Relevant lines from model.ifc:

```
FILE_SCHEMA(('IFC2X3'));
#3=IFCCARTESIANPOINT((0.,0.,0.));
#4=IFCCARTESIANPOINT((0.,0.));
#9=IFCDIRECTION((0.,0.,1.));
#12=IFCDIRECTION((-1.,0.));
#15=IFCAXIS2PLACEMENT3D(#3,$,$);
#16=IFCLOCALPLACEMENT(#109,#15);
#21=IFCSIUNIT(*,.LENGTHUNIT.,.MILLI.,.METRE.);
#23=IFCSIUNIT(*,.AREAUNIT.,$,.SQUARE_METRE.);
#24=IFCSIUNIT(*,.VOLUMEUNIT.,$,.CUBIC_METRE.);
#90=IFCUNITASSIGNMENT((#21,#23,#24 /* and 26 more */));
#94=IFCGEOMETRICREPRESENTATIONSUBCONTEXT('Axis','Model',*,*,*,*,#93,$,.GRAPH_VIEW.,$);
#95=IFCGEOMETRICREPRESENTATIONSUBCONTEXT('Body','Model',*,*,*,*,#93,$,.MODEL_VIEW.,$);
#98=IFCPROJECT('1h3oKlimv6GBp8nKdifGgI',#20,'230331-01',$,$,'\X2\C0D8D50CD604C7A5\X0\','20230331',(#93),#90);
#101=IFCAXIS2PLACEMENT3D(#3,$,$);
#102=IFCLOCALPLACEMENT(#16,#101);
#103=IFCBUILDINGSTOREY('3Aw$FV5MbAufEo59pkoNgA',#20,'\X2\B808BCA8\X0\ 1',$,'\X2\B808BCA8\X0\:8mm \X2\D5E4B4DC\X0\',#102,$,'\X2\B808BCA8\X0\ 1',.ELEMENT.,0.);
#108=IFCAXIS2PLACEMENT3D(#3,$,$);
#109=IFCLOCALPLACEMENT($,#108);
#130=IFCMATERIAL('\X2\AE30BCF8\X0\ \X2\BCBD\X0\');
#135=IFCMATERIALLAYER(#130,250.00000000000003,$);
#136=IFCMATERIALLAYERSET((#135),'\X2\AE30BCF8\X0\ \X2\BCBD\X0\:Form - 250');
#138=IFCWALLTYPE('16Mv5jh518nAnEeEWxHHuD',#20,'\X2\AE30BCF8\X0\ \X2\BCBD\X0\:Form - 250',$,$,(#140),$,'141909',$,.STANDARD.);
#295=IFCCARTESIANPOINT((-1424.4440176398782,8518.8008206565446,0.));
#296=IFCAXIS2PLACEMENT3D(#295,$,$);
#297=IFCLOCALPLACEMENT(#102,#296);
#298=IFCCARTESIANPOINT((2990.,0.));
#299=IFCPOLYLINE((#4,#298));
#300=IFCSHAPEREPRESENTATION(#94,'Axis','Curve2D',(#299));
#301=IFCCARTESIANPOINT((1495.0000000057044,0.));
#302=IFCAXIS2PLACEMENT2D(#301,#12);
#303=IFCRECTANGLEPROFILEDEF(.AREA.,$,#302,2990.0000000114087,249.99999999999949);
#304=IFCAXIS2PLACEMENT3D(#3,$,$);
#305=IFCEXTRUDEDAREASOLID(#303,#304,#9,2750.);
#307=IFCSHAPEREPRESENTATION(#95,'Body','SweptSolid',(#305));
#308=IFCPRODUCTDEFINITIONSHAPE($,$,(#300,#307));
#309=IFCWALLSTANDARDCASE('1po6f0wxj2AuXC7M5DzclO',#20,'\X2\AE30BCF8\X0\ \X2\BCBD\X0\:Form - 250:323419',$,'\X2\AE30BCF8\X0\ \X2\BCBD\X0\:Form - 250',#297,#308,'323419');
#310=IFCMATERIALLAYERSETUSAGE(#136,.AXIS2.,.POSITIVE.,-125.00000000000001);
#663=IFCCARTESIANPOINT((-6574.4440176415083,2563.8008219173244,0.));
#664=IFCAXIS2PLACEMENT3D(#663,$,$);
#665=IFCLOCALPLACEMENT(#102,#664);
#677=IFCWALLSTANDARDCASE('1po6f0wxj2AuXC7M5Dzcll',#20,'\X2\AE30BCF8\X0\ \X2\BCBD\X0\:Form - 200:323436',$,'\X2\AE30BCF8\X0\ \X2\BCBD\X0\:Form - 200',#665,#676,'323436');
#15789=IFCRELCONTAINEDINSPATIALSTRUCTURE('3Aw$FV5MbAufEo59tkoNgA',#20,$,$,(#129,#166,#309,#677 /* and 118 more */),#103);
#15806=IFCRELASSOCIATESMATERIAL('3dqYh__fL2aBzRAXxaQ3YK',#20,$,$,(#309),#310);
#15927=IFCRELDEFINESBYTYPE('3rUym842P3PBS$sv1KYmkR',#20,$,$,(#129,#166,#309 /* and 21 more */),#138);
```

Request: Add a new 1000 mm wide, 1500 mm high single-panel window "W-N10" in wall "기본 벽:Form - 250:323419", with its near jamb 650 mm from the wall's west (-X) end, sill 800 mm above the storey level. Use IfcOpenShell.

```python
import numpy as np
import ifcopenshell
import ifcopenshell.api.feature
import ifcopenshell.api.geometry
import ifcopenshell.api.root
import ifcopenshell.api.spatial
import ifcopenshell.api.type
import ifcopenshell.geom
import ifcopenshell.util.element
import ifcopenshell.util.placement
import ifcopenshell.util.representation
import ifcopenshell.util.shape
import ifcopenshell.util.unit

model = ifcopenshell.open("model.ifc")
unit_scale = ifcopenshell.util.unit.calculate_unit_scale(model)
settings = ifcopenshell.geom.settings()


def volume(element):
    """Net volume in cubic metres, openings subtracted."""
    shape = ifcopenshell.geom.create_shape(settings, element)
    return ifcopenshell.util.shape.get_volume(shape.geometry)


wall = model.by_guid("1po6f0wxj2AuXC7M5DzclO")
storey = ifcopenshell.util.element.get_container(wall, ifc_class="IfcBuildingStorey")
context = ifcopenshell.util.representation.get_context(model, "Model", "Body", "MODEL_VIEW")
before = volume(wall)

width, height, from_end, sill = 1, 1.5, 0.65, 0.8  # metres

# The wall runs along its own X axis, and the end named is its -X end.
wall_shape = ifcopenshell.geom.create_shape(settings, wall)
x, y, z = ifcopenshell.util.shape.get_vertices(wall_shape.geometry).T
start = x.min() + from_end
face, thickness = float(y.min()), float(y.max() - y.min())
wall_matrix = ifcopenshell.util.placement.get_local_placement(wall.ObjectPlacement)
level = ifcopenshell.util.placement.get_local_placement(storey.ObjectPlacement)[2, 3]


def in_wall(x, y):
    """Placement at x, y metres in the wall's axes, at sill height."""
    matrix = wall_matrix.copy()
    matrix[:, 3] = wall_matrix @ np.array([x / unit_scale, y / unit_scale, 0.0, 1.0])
    matrix[2, 3] = level + sill / unit_scale
    return matrix


# Opening: a box that overshoots both wall faces by 50 mm.
opening = ifcopenshell.api.root.create_entity(model, ifc_class="IfcOpeningElement")
box = ifcopenshell.api.geometry.add_wall_representation(
    model, context=context, length=width, height=height, thickness=thickness + 0.1
)
ifcopenshell.api.geometry.assign_representation(model, product=opening, representation=box)
ifcopenshell.api.geometry.edit_object_placement(model, product=opening, matrix=in_wall(start, face - 0.05), is_si=False)
ifcopenshell.api.feature.add_feature(model, feature=opening, element=wall)

window = ifcopenshell.api.root.create_entity(model, ifc_class="IfcWindow", name="W-N10")
window.OverallWidth, window.OverallHeight = width / unit_scale, height / unit_scale
body = ifcopenshell.api.geometry.add_window_representation(
    model,
    context=context,
    overall_width=window.OverallWidth,
    overall_height=window.OverallHeight,
    partition_type="SINGLE_PANEL",
)
ifcopenshell.api.geometry.assign_representation(model, product=window, representation=body)
ifcopenshell.api.spatial.assign_container(model, products=[window], relating_structure=storey)
fills = ifcopenshell.api.feature.add_filling(model, opening=opening, element=window)
fills.OwnerHistory = window.OwnerHistory  # required in IFC2X3

# IFC2X3 keeps the operation on the window style.
style = ifcopenshell.api.root.create_entity(model, ifc_class="IfcWindowStyle", name="W-N10")
style.OperationType, style.ConstructionType = "SINGLE_PANEL", "NOTDEFINED"
style.ParameterTakesPrecedence = style.Sizeable = False
ifcopenshell.api.type.assign_type(model, related_objects=[window], relating_type=style)

# Centre the window in the wall's thickness.
ifcopenshell.api.geometry.edit_object_placement(model, product=window, matrix=in_wall(start, face), is_si=False)
window_shape = ifcopenshell.geom.create_shape(settings, window)
depth = ifcopenshell.util.shape.get_vertices(window_shape.geometry)[:, 1]
offset = face + thickness / 2 - (depth.min() + depth.max()) / 2
ifcopenshell.api.geometry.edit_object_placement(model, product=window, matrix=in_wall(start, offset), is_si=False)

after = volume(wall)

print(f"wall volume {before:.3f} -> {after:.3f} m3")

model.write("model_v2.ifc")
```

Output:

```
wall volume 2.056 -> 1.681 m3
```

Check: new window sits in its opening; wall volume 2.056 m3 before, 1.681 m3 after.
